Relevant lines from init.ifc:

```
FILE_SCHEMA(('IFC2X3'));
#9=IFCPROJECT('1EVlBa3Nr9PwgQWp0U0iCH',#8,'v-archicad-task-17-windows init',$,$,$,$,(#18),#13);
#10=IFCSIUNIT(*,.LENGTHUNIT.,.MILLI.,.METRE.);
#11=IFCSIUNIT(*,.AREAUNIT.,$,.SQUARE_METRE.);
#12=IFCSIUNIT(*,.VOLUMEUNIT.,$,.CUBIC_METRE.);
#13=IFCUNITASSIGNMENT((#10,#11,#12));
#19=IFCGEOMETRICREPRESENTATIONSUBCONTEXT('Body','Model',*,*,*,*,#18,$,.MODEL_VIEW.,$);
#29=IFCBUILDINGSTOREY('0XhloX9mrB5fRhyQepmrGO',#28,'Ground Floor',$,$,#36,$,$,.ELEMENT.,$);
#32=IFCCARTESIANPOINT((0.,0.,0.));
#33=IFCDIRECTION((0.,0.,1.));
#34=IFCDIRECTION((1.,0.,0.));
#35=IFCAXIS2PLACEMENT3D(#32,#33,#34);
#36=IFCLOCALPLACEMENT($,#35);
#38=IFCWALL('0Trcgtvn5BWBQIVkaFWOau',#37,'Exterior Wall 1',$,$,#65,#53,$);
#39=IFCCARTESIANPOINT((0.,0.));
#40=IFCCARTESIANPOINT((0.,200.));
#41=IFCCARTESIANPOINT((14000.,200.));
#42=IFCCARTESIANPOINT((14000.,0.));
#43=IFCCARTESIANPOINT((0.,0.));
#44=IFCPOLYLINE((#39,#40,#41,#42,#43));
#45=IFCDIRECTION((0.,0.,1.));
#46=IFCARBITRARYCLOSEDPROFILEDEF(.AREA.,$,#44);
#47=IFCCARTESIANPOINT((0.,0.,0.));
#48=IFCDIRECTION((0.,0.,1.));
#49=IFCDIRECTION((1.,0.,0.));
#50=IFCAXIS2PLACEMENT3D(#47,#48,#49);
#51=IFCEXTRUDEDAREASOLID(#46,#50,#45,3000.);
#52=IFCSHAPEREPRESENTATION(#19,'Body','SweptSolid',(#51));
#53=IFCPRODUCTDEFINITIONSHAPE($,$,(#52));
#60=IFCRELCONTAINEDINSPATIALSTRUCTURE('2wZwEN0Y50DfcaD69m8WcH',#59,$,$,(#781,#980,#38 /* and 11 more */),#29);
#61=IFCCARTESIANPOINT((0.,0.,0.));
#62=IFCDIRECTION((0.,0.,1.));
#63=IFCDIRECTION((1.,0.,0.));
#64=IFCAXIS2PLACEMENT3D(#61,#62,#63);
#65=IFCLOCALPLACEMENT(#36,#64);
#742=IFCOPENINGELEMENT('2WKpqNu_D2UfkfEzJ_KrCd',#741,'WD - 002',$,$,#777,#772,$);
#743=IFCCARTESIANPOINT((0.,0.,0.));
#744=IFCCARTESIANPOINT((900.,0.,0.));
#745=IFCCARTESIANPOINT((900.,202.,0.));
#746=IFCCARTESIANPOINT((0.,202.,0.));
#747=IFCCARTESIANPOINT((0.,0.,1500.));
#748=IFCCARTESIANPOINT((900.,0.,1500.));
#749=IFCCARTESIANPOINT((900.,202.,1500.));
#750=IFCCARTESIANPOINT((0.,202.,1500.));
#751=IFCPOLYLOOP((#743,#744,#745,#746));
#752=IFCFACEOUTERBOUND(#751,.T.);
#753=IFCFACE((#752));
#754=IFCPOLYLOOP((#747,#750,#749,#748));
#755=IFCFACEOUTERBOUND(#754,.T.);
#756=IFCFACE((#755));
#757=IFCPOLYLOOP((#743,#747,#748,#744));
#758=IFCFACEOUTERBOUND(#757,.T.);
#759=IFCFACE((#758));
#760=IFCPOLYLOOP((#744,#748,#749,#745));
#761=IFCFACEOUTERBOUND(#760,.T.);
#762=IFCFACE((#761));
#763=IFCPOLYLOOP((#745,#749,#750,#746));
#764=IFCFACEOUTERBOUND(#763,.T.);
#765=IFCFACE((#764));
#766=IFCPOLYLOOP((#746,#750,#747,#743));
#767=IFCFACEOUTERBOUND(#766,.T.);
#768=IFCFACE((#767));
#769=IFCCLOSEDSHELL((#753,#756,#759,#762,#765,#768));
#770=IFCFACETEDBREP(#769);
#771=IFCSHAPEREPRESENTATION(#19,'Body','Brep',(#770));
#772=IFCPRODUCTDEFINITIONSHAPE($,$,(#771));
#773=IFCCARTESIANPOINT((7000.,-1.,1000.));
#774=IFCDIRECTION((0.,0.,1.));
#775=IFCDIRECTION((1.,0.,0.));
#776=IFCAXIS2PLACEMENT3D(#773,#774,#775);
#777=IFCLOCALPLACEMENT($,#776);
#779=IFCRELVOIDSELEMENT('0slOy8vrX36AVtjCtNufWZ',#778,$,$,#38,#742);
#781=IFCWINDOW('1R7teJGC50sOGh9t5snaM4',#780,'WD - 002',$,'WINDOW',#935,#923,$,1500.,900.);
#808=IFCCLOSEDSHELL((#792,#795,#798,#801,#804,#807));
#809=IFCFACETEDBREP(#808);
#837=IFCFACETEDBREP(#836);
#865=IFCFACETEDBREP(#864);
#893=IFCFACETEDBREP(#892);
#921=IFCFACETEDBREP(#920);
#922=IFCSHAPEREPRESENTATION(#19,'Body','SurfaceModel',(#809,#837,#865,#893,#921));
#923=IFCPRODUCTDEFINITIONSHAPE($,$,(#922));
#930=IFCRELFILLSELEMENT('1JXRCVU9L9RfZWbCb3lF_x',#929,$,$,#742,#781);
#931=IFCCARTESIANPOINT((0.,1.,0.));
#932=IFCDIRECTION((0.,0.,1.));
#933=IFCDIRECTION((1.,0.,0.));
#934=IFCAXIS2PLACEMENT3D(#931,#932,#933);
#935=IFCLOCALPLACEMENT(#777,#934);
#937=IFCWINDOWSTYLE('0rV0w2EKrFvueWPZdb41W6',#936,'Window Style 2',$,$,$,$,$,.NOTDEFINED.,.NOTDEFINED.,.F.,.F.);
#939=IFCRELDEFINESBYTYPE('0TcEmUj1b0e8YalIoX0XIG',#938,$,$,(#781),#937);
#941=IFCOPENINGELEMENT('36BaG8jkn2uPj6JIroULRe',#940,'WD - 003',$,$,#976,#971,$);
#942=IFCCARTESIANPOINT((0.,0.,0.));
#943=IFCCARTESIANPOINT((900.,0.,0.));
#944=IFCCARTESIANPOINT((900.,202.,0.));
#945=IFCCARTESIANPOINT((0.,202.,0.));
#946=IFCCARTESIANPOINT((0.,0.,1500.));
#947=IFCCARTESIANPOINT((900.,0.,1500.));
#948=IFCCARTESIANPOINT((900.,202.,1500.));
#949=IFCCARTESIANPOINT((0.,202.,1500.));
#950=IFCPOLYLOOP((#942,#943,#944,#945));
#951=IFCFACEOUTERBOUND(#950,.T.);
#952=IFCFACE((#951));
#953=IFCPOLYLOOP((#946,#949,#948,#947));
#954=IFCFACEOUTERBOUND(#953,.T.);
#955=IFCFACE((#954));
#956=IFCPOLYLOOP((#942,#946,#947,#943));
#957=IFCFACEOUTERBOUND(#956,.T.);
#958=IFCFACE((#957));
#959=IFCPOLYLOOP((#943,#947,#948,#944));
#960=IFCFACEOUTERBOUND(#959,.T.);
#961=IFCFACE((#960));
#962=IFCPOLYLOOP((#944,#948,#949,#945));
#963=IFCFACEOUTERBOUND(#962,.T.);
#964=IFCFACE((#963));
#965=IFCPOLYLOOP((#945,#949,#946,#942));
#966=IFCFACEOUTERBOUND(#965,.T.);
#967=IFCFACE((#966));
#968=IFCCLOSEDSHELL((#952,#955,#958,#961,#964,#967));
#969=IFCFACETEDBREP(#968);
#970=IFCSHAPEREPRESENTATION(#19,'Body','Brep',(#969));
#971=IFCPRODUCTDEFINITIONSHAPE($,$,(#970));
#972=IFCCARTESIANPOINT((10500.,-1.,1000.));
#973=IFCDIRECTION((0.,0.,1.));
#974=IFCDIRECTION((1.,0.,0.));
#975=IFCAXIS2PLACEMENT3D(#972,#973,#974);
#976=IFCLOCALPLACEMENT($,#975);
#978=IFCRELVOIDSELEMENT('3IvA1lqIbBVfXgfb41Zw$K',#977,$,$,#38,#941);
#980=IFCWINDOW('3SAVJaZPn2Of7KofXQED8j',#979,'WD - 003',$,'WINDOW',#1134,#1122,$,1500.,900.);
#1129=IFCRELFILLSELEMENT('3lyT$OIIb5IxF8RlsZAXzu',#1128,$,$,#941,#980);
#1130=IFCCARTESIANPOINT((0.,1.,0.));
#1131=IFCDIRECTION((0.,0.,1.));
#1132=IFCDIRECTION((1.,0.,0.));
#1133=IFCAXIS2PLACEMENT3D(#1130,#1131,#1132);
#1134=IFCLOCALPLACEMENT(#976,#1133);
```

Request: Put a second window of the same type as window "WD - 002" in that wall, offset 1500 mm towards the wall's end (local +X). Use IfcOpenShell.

```python
import ifcopenshell
import ifcopenshell.api.feature
import ifcopenshell.api.geometry
import ifcopenshell.api.root
import ifcopenshell.geom
import ifcopenshell.util.element
import ifcopenshell.util.placement
import ifcopenshell.util.shape
import ifcopenshell.util.unit

model = ifcopenshell.open("init.ifc")
unit_scale = ifcopenshell.util.unit.calculate_unit_scale(model)
settings = ifcopenshell.geom.settings()


def volume(element):
    """Net volume in cubic metres, openings subtracted."""
    shape = ifcopenshell.geom.create_shape(settings, element)
    return ifcopenshell.util.shape.get_volume(shape.geometry)


window = model.by_id(781)
opening = window.FillsVoids[0].RelatingOpeningElement
wall = opening.VoidsElements[0].RelatingBuildingElement
before = volume(wall)
shift = ifcopenshell.util.placement.get_local_placement(wall.ObjectPlacement)[:3, 0] * 1.5 / unit_scale

# copy_class copies the void relationship, type, container and properties, but no geometry.
new_opening = ifcopenshell.api.root.copy_class(model, product=opening)
new_opening.Representation = ifcopenshell.util.element.copy_deep(
    model, opening.Representation, exclude=["IfcGeometricRepresentationContext", "IfcRepresentationMap"]
)
new_window = ifcopenshell.api.root.copy_class(model, product=window)
new_window.Representation = ifcopenshell.util.element.copy_deep(
    model, window.Representation, exclude=["IfcGeometricRepresentationContext", "IfcRepresentationMap"]
)
fills = ifcopenshell.api.feature.add_filling(model, opening=new_opening, element=new_window)
fills.OwnerHistory = new_window.OwnerHistory  # required in IFC2X3

for old, new in ((opening, new_opening), (window, new_window)):
    matrix = ifcopenshell.util.placement.get_local_placement(old.ObjectPlacement)
    matrix[:3, 3] += shift
    ifcopenshell.api.geometry.edit_object_placement(model, product=new, matrix=matrix, is_si=False)

after = volume(wall)

print(f"wall volume {before:.3f} -> {after:.3f} m3")

model.write("init-out.ifc")
```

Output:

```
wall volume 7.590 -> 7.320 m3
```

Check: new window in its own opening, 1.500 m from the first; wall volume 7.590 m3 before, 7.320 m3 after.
